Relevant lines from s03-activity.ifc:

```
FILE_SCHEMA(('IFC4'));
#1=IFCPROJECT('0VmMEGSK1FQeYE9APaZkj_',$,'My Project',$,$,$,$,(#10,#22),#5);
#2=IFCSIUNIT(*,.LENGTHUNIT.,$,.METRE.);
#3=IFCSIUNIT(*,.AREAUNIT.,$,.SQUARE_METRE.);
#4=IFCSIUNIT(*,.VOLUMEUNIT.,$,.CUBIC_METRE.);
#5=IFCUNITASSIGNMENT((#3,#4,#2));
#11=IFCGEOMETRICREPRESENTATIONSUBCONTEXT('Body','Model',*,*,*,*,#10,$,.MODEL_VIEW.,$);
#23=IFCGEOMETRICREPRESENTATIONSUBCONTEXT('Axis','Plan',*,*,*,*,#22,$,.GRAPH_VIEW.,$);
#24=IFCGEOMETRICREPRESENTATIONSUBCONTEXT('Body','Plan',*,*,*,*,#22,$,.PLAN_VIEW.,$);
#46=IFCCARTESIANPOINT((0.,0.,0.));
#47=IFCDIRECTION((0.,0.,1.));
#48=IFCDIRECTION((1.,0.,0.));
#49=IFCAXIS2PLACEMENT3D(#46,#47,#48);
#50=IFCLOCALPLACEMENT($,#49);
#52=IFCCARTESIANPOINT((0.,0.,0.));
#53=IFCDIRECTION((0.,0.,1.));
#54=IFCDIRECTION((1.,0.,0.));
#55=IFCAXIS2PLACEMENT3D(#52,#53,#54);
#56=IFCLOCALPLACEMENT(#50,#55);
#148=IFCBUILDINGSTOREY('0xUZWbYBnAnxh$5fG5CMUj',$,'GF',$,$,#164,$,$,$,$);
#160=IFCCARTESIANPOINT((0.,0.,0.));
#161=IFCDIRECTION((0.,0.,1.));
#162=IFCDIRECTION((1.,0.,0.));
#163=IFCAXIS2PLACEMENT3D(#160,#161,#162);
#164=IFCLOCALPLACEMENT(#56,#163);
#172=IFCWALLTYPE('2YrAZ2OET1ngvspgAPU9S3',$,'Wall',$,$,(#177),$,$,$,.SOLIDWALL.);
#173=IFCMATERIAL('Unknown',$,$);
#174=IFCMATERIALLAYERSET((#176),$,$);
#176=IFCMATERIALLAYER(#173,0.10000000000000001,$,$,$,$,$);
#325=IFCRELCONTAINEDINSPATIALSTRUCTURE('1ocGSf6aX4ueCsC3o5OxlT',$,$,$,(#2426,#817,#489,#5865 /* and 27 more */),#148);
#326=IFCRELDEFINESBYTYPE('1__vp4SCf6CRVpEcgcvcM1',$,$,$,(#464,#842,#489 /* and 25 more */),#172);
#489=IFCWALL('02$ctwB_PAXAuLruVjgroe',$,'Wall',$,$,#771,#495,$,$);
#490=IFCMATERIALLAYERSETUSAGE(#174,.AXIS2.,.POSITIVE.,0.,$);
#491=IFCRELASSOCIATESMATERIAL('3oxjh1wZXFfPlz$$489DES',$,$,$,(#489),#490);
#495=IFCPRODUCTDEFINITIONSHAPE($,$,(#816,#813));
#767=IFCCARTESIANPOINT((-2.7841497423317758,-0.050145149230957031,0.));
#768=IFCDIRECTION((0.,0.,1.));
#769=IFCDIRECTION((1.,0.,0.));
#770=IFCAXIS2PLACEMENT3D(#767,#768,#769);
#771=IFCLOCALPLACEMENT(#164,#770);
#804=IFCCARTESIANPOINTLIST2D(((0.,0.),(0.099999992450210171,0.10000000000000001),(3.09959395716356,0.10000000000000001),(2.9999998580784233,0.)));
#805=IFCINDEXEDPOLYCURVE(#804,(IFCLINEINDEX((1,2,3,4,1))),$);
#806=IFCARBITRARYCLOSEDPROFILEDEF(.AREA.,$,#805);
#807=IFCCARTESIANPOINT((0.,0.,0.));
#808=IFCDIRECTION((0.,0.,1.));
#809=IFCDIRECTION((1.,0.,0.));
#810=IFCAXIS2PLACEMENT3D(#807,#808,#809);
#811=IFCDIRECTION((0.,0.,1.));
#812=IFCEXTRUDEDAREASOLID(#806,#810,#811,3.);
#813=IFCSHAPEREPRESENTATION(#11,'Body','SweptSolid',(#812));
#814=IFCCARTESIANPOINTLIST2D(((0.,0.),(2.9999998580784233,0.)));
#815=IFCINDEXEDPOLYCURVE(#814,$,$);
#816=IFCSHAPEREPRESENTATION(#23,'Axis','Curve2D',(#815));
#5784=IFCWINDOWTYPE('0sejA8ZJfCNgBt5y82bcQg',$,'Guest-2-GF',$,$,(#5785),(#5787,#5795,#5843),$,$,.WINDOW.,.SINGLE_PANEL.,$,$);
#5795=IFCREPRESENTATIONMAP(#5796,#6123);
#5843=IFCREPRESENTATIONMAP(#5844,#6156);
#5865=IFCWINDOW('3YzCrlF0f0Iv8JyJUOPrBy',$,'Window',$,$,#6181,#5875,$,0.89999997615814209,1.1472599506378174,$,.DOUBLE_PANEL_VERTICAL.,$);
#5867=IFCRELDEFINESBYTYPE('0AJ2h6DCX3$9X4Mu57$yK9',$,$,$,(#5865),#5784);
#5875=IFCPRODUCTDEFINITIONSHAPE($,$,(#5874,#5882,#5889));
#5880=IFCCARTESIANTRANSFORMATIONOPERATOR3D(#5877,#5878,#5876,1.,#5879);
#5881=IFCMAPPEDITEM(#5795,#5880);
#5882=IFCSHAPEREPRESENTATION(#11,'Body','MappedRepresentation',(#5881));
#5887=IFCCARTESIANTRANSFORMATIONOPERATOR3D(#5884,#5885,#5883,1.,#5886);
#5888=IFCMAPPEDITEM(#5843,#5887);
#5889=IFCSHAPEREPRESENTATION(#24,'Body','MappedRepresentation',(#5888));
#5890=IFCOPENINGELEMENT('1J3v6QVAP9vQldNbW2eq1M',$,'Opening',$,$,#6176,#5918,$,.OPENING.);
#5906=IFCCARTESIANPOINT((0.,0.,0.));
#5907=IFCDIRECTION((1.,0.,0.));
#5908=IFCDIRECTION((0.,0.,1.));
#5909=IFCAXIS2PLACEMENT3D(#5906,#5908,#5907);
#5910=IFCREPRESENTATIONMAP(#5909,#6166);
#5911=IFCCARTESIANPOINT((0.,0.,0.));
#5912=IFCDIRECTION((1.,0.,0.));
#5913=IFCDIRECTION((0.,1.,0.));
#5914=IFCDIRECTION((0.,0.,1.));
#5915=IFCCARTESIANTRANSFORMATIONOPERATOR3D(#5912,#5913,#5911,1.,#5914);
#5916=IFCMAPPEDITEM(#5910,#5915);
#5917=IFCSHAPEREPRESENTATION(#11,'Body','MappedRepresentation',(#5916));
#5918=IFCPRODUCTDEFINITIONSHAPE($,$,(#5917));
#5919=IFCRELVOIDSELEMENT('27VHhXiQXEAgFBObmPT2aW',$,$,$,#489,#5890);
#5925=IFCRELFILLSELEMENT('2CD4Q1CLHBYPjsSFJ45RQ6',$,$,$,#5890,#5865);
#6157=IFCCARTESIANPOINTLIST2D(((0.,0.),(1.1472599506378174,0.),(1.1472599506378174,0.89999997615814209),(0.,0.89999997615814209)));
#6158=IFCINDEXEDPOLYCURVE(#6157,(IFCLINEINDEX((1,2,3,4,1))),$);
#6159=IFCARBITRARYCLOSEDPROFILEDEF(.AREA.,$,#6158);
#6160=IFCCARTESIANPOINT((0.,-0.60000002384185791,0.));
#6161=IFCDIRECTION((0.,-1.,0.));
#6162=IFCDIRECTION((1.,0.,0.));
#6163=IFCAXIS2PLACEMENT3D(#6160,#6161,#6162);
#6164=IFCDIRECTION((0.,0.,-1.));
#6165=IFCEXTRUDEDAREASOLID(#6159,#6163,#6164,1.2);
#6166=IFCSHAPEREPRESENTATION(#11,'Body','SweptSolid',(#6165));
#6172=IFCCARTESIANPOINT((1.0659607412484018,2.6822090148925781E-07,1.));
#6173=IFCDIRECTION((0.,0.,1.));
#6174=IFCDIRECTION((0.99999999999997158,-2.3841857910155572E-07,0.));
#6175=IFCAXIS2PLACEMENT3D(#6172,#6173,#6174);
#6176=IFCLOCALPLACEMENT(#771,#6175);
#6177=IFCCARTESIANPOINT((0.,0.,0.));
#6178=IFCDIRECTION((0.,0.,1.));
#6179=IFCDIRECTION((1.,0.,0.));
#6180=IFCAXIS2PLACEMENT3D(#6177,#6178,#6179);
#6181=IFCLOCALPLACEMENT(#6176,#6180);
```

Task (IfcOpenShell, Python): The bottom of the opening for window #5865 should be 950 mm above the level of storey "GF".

```python
import numpy as np
import ifcopenshell
import ifcopenshell.api.geometry
import ifcopenshell.geom
import ifcopenshell.util.element
import ifcopenshell.util.placement
import ifcopenshell.util.shape
import ifcopenshell.util.unit

model = ifcopenshell.open("s03-activity.ifc")
unit_scale = ifcopenshell.util.unit.calculate_unit_scale(model)

window = model.by_guid("3YzCrlF0f0Iv8JyJUOPrBy")
opening = window.FillsVoids[0].RelatingOpeningElement
storey = ifcopenshell.util.element.get_container(window, ifc_class="IfcBuildingStorey")
level = ifcopenshell.util.placement.get_local_placement(storey.ObjectPlacement)[2, 3]

# The opening's origin need not be at the sill, so measure its lowest point.
shape = ifcopenshell.geom.create_shape(ifcopenshell.geom.settings(), opening)
bottom = ifcopenshell.util.shape.get_shape_bottom_elevation(shape, shape.geometry) / unit_scale
dz = level + 0.95 - bottom

shift = np.array([0.0, 0.0, dz])
# The window is placed relative to its opening, so it follows when the opening moves.
matrix = ifcopenshell.util.placement.get_local_placement(opening.ObjectPlacement)
matrix[:3, 3] += shift
ifcopenshell.api.geometry.edit_object_placement(
    model, product=opening, matrix=matrix, is_si=False, should_transform_children=True
)

print(f"moved by {dz * unit_scale:+.3f} m")

model.write("s03-activity_rev.ifc")
```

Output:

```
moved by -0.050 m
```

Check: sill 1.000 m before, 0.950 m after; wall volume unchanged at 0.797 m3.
